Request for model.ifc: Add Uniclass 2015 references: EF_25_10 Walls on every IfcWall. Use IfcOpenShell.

First a look at what the model holds.

```python
import ifcopenshell

model = ifcopenshell.open("model.ifc")
print(model.schema)
print("classifications:", [c.Name for c in model.by_type("IfcClassification")])
for ifc_class in ("IfcDoor", "IfcRoof", "IfcStair", "IfcWall", "IfcWindow"):
    print(ifc_class, len(model.by_type(ifc_class)))
```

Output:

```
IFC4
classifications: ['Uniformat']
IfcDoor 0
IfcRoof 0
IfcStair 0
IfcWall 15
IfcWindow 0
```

```python
import ifcopenshell
import ifcopenshell.api.classification

model = ifcopenshell.open("model.ifc")

system = ifcopenshell.api.classification.add_classification(model, classification="Uniclass 2015")

codes = {
    "IfcWall": ("EF_25_10", "Walls"),
}
for ifc_class, (code, name) in codes.items():
    products = model.by_type(ifc_class)
    ifcopenshell.api.classification.add_reference(
        model, products=products, classification=system, identification=code, name=name
    )
    print(code, len(products))

model.write("model-out.ifc")
```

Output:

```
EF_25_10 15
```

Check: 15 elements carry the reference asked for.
